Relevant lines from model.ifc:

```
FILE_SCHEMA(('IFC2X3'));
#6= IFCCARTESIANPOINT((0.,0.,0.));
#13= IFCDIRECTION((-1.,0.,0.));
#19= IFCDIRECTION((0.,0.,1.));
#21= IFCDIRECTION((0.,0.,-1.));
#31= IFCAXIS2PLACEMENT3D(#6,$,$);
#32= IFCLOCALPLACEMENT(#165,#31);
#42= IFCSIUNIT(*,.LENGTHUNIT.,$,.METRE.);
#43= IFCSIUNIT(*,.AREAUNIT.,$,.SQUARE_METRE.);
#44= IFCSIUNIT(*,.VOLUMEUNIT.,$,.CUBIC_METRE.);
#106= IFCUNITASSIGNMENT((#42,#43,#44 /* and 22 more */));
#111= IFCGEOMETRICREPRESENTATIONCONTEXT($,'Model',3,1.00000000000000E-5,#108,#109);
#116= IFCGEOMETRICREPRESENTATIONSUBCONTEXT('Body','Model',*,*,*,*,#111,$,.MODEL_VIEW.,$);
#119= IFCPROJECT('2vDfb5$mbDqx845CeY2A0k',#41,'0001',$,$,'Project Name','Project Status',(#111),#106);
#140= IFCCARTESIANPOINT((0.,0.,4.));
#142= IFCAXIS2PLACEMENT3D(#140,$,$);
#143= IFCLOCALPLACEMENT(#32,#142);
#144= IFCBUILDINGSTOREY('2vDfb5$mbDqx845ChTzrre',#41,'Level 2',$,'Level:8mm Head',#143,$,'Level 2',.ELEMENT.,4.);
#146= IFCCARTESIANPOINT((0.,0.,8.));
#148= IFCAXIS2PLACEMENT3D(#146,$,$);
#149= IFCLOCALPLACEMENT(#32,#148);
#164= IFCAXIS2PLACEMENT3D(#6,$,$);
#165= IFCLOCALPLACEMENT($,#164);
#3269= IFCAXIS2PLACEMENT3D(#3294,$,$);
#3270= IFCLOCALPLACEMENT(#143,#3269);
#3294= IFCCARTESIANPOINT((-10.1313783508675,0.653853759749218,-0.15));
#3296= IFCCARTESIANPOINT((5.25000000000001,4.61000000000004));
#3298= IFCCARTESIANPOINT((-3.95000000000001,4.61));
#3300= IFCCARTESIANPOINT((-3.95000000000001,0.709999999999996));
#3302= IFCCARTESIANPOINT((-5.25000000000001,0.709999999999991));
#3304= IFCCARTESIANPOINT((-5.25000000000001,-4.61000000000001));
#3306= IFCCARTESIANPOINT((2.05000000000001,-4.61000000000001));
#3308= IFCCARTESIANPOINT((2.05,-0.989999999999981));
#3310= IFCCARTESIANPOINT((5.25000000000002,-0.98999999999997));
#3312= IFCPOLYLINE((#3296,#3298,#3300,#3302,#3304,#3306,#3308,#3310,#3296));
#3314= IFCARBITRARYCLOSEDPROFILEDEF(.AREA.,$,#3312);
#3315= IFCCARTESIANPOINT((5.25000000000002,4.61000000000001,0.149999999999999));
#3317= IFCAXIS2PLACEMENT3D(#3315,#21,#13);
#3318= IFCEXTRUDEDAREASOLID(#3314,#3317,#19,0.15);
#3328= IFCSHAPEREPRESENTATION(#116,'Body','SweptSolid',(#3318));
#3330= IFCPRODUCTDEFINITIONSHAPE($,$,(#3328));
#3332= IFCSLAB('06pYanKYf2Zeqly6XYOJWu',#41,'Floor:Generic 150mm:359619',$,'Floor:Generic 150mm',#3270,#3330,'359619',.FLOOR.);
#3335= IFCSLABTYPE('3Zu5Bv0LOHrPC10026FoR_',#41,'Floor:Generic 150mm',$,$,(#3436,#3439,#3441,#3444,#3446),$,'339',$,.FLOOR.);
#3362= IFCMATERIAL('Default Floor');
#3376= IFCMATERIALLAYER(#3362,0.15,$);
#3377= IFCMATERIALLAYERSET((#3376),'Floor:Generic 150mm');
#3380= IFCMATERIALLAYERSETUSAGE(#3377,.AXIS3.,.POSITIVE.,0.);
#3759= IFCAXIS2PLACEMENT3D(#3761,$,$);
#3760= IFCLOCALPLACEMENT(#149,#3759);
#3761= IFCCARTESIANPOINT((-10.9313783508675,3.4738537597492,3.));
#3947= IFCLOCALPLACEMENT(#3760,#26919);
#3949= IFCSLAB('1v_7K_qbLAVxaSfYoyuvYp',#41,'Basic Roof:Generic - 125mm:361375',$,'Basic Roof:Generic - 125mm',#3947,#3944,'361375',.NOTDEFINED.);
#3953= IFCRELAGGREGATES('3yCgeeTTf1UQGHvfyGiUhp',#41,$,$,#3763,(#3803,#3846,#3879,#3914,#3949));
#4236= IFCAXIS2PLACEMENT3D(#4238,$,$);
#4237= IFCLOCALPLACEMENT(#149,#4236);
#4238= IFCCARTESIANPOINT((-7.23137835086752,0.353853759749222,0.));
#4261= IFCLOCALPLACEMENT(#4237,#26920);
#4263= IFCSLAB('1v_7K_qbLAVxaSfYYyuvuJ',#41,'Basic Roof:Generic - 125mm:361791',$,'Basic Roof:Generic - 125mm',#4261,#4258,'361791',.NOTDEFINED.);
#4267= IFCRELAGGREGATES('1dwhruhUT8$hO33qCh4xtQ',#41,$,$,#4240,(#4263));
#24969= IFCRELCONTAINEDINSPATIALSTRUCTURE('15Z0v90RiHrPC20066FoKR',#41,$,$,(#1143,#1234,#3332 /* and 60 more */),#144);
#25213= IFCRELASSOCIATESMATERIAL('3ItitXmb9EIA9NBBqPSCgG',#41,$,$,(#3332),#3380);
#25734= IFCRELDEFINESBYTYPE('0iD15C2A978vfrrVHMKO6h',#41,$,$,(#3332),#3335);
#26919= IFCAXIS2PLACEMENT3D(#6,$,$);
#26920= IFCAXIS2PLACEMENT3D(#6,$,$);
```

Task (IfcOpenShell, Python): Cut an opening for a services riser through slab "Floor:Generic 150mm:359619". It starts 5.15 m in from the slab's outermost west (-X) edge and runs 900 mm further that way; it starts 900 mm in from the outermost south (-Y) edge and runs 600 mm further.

```python
import numpy as np
import ifcopenshell
import ifcopenshell.api.feature
import ifcopenshell.api.geometry
import ifcopenshell.api.root
import ifcopenshell.geom
import ifcopenshell.util.placement
import ifcopenshell.util.representation
import ifcopenshell.util.shape
import ifcopenshell.util.unit

model = ifcopenshell.open("model.ifc")
unit_scale = ifcopenshell.util.unit.calculate_unit_scale(model)
settings = ifcopenshell.geom.settings()


def volume(element):
    """Net volume in cubic metres, openings subtracted."""
    shape = ifcopenshell.geom.create_shape(settings, element)
    return ifcopenshell.util.shape.get_volume(shape.geometry)


slab = model.by_guid("06pYanKYf2Zeqly6XYOJWu")
before = volume(slab)

# Extent in the slab's own axes, in metres. The edges named are its -X and -Y sides.
slab_shape = ifcopenshell.geom.create_shape(settings, slab)
vertices = ifcopenshell.util.shape.get_vertices(slab_shape.geometry)
x_min, y_min, bottom = vertices.min(axis=0)
top = vertices[:, 2].max()

opening = ifcopenshell.api.root.create_entity(model, ifc_class="IfcOpeningElement", name="Services riser opening")
context = ifcopenshell.util.representation.get_context(model, "Model", "Body", "MODEL_VIEW")
width, depth = 0.9, 0.6
outline = [(0.0, 0.0), (width, 0.0), (width, depth), (0.0, depth), (0.0, 0.0)]
# Overshoot both faces by 50 mm so the cut is clean.
shape = ifcopenshell.api.geometry.add_slab_representation(
    model, context=context, depth=top - bottom + 0.1, polyline=outline
)
ifcopenshell.api.geometry.assign_representation(model, product=opening, representation=shape)

matrix = ifcopenshell.util.placement.get_local_placement(slab.ObjectPlacement)
matrix[:, 3] = matrix @ np.append(np.array([x_min + 5.15, y_min + 0.9, bottom - 0.05]) / unit_scale, 1.0)
ifcopenshell.api.geometry.edit_object_placement(model, product=opening, matrix=matrix, is_si=False)
ifcopenshell.api.feature.add_feature(model, feature=opening, element=slab)

after = volume(slab)

print(f"slab volume {before:.3f} -> {after:.3f} m3")

model.write("model-out.ifc")
```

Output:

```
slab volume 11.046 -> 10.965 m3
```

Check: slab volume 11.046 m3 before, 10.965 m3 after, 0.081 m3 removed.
